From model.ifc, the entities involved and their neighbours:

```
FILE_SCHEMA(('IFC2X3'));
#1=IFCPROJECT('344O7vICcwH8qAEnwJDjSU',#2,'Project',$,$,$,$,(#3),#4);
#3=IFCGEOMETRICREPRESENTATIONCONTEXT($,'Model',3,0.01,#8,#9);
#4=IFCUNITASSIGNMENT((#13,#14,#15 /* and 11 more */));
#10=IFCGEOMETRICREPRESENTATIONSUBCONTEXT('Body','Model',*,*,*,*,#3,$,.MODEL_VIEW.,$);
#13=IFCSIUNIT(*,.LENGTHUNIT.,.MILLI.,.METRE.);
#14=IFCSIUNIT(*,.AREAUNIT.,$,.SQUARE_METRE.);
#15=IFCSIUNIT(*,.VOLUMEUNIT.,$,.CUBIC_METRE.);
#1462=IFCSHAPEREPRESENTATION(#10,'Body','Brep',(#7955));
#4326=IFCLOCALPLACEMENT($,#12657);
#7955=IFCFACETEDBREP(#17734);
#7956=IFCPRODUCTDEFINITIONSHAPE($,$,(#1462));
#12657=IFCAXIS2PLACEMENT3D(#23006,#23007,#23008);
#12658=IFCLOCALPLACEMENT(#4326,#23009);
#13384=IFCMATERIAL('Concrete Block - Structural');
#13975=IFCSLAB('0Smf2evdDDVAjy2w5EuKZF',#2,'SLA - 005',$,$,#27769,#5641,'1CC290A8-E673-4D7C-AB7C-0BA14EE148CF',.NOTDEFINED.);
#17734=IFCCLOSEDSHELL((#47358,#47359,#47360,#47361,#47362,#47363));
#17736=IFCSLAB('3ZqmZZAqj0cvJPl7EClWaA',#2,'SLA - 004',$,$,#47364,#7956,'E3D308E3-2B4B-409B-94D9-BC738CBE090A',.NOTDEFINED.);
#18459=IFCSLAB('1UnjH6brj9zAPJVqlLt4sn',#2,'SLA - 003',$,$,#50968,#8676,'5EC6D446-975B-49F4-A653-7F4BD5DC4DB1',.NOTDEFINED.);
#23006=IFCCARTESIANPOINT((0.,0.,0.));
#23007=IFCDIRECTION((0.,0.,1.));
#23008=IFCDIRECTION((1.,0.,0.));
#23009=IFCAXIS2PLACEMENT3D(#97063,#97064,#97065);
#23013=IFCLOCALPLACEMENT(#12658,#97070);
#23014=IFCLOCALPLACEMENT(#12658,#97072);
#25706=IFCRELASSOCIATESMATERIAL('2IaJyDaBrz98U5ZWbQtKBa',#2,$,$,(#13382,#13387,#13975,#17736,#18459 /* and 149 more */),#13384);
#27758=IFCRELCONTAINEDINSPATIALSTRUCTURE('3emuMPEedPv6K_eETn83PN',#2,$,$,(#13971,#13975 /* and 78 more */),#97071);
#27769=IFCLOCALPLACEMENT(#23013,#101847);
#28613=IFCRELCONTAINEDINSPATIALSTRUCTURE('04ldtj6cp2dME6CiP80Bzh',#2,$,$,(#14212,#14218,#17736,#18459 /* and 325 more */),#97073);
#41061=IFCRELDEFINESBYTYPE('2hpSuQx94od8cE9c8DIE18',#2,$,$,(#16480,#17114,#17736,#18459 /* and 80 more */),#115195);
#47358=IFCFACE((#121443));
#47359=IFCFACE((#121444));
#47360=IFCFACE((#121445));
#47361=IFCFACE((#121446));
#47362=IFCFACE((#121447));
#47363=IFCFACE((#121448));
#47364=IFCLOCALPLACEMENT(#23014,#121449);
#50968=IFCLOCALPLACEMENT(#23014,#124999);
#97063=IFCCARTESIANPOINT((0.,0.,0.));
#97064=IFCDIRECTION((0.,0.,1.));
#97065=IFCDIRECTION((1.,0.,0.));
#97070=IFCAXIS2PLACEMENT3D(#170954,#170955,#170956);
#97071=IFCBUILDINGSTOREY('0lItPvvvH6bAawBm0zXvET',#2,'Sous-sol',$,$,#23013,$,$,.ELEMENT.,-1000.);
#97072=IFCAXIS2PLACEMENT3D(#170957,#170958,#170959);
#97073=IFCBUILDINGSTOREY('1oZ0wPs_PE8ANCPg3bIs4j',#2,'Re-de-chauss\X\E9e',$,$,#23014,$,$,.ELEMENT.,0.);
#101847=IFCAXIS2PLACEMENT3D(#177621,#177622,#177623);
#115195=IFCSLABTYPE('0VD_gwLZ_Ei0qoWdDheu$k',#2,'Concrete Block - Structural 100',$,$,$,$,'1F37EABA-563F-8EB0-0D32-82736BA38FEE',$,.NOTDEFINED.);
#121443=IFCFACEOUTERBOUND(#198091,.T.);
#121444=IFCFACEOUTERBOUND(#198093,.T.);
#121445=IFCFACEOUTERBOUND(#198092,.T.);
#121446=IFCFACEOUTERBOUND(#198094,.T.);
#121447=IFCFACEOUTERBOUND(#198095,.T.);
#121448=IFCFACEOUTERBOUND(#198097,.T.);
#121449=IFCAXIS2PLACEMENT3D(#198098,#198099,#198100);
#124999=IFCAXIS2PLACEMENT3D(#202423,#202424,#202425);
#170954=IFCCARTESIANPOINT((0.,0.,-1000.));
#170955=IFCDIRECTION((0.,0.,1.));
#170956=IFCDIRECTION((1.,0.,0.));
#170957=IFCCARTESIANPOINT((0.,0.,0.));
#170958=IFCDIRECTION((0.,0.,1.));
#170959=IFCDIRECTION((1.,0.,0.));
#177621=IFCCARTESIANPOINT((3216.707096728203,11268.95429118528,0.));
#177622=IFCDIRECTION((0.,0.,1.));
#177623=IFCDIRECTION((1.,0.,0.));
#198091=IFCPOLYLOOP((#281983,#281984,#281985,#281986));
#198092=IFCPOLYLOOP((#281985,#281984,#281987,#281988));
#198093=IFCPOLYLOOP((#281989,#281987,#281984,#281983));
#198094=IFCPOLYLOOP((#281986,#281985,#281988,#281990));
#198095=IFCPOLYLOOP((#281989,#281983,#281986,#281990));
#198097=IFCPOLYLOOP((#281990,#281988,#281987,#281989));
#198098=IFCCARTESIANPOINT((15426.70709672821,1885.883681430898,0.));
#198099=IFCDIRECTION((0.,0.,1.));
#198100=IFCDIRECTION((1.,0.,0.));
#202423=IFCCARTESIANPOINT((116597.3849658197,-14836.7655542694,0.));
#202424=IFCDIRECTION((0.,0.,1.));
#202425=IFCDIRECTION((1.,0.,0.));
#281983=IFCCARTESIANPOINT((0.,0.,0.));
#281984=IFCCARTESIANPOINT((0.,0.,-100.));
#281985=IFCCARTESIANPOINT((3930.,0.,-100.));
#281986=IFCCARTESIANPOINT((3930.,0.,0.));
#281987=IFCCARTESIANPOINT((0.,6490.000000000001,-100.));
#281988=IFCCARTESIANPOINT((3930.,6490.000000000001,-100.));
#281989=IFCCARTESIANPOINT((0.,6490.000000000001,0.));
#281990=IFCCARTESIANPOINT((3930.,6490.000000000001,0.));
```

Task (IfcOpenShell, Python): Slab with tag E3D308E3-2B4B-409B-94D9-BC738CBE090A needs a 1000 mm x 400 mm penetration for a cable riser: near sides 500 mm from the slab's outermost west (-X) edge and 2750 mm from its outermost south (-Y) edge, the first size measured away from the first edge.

```python
import numpy as np
import ifcopenshell
import ifcopenshell.api.feature
import ifcopenshell.api.geometry
import ifcopenshell.api.root
import ifcopenshell.geom
import ifcopenshell.util.placement
import ifcopenshell.util.representation
import ifcopenshell.util.shape
import ifcopenshell.util.unit

model = ifcopenshell.open("model.ifc")
unit_scale = ifcopenshell.util.unit.calculate_unit_scale(model)
settings = ifcopenshell.geom.settings()


def volume(element):
    """Net volume in cubic metres, openings subtracted."""
    shape = ifcopenshell.geom.create_shape(settings, element)
    return ifcopenshell.util.shape.get_volume(shape.geometry)


slab = model.by_guid("3ZqmZZAqj0cvJPl7EClWaA")
before = volume(slab)

# Extent in the slab's own axes, in metres. The edges named are its -X and -Y sides.
slab_shape = ifcopenshell.geom.create_shape(settings, slab)
vertices = ifcopenshell.util.shape.get_vertices(slab_shape.geometry)
x_min, y_min, bottom = vertices.min(axis=0)
top = vertices[:, 2].max()

opening = ifcopenshell.api.root.create_entity(model, ifc_class="IfcOpeningElement", name="Cable riser opening")
context = ifcopenshell.util.representation.get_context(model, "Model", "Body", "MODEL_VIEW")
width, depth = 1, 0.4
outline = [(0.0, 0.0), (width, 0.0), (width, depth), (0.0, depth), (0.0, 0.0)]
# Overshoot both faces by 50 mm so the cut is clean.
shape = ifcopenshell.api.geometry.add_slab_representation(
    model, context=context, depth=top - bottom + 0.1, polyline=outline
)
ifcopenshell.api.geometry.assign_representation(model, product=opening, representation=shape)

matrix = ifcopenshell.util.placement.get_local_placement(slab.ObjectPlacement)
matrix[:, 3] = matrix @ np.append(np.array([x_min + 0.5, y_min + 2.75, bottom - 0.05]) / unit_scale, 1.0)
ifcopenshell.api.geometry.edit_object_placement(model, product=opening, matrix=matrix, is_si=False)
ifcopenshell.api.feature.add_feature(model, feature=opening, element=slab)

after = volume(slab)

print(f"slab volume {before:.3f} -> {after:.3f} m3")

model.write("model_updated.ifc")
```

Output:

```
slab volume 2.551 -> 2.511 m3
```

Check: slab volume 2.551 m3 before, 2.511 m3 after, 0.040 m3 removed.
